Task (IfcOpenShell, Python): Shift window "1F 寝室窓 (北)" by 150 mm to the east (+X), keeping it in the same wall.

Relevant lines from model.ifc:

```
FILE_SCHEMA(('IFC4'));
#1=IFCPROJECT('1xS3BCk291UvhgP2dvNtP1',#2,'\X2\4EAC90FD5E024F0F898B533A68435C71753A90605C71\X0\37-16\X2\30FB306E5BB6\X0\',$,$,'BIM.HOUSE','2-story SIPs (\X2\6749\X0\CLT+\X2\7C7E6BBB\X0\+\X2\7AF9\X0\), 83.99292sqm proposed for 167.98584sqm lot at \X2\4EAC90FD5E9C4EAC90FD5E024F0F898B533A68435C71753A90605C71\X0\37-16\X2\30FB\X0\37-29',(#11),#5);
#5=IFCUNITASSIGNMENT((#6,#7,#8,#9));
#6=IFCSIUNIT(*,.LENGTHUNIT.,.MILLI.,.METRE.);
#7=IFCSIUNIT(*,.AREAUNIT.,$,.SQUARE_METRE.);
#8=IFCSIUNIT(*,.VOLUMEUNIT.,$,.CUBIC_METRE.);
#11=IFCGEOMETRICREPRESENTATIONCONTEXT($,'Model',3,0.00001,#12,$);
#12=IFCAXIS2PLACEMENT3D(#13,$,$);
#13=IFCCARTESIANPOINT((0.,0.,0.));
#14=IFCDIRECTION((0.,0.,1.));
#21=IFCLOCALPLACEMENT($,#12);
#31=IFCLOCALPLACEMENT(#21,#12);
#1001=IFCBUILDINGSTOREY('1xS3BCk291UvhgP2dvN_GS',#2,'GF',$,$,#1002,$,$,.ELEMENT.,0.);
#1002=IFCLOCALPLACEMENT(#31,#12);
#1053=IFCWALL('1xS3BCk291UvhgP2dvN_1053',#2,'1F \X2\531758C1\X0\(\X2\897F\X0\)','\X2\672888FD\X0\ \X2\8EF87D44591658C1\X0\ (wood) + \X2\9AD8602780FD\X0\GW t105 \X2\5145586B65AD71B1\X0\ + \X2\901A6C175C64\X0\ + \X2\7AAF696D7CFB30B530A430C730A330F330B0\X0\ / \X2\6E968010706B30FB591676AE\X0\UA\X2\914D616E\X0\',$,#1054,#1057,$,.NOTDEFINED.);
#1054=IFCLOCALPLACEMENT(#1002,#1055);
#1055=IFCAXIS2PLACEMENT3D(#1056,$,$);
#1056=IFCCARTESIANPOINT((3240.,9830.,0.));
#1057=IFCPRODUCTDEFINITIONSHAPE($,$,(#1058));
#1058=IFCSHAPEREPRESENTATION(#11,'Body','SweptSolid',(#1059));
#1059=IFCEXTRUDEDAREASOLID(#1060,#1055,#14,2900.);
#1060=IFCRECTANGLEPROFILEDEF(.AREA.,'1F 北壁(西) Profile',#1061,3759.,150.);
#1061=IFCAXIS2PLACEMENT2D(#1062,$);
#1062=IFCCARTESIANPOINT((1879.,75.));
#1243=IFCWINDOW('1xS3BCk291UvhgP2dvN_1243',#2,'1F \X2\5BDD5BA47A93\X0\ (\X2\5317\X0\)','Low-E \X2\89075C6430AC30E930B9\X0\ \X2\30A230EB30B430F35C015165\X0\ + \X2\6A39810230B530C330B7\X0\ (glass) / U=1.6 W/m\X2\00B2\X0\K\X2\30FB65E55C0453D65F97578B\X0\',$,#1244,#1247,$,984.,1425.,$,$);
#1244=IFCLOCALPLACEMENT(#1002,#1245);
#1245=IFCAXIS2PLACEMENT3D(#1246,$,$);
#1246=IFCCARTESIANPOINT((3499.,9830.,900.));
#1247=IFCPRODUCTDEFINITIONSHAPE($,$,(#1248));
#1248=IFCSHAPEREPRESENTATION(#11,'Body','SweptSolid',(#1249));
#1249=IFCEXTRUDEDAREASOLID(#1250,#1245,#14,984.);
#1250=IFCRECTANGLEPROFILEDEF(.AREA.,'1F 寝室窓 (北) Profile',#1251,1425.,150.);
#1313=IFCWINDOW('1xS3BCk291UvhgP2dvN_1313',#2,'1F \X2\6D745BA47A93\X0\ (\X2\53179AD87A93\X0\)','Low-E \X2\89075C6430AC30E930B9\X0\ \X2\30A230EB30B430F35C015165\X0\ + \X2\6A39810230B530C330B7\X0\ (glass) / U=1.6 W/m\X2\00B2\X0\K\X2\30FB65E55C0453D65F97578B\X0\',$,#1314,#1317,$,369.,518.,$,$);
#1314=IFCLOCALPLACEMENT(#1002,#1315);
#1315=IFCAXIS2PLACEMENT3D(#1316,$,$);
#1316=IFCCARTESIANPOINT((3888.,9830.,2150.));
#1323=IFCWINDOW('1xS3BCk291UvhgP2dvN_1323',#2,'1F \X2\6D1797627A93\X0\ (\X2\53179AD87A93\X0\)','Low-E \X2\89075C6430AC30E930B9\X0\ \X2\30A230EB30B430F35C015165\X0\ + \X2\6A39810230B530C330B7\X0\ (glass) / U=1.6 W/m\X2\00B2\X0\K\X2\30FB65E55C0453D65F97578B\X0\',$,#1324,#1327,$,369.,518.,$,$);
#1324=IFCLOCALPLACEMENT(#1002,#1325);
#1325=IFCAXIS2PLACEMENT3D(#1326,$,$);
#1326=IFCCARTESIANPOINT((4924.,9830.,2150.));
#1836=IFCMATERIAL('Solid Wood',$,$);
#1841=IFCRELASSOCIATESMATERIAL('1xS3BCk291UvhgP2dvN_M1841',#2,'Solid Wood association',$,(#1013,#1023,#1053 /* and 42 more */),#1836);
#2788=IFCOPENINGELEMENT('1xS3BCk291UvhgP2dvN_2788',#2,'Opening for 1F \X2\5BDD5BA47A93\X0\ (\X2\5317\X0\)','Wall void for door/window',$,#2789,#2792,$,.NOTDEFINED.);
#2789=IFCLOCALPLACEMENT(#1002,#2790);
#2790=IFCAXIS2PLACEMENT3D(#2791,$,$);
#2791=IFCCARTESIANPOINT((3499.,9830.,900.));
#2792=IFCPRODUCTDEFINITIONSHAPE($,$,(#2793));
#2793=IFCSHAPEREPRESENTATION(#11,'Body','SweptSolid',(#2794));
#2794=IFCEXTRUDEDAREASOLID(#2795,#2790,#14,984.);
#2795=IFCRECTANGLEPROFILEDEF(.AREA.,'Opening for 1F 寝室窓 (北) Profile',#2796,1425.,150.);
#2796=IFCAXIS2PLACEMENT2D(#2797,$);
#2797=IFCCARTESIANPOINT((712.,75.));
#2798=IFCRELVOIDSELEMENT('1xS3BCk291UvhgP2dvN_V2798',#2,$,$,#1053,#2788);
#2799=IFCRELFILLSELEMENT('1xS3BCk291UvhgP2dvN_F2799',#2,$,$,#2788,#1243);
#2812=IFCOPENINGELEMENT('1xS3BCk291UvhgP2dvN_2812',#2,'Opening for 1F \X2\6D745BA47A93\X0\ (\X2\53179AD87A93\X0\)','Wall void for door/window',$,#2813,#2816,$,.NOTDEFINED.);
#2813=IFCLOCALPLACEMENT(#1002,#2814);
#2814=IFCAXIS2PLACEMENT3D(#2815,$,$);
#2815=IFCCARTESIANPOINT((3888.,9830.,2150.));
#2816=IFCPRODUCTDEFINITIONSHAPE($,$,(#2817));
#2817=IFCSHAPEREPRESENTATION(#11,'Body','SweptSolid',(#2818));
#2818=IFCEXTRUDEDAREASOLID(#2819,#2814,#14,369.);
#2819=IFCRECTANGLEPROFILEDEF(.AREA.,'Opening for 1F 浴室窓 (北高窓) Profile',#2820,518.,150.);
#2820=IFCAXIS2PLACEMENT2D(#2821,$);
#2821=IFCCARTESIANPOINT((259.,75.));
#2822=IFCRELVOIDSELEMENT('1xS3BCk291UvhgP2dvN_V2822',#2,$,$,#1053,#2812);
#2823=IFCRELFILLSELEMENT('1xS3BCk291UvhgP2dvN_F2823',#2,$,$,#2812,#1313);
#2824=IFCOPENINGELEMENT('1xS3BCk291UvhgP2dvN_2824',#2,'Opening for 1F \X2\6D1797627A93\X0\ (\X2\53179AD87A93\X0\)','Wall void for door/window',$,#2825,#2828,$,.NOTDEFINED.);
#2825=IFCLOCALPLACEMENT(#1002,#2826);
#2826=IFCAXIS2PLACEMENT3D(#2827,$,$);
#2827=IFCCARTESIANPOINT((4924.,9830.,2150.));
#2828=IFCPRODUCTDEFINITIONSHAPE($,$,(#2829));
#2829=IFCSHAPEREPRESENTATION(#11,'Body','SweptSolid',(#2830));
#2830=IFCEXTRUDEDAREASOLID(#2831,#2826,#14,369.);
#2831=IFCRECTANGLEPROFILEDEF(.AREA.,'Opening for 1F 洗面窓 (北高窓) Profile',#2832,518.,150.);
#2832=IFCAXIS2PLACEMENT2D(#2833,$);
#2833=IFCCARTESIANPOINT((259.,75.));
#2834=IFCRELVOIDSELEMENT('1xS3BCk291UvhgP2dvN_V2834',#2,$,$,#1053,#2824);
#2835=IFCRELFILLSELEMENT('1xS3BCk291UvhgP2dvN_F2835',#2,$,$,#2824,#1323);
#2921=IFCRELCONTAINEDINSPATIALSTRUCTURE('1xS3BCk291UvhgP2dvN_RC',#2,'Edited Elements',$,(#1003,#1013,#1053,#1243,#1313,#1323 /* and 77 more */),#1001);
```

```python
import ifcopenshell
import ifcopenshell.api.geometry
import ifcopenshell.util.placement

model = ifcopenshell.open("model.ifc")

window = model.by_guid("1xS3BCk291UvhgP2dvN_1243")
opening = window.FillsVoids[0].RelatingOpeningElement
wall = opening.VoidsElements[0].RelatingBuildingElement

wall_matrix = ifcopenshell.util.placement.get_local_placement(wall.ObjectPlacement)
shift = wall_matrix[:3, 0] * 150.0
before = ifcopenshell.util.placement.get_local_placement(window.ObjectPlacement)[:3, 3].copy()

# The window is not placed relative to its opening, so move both.
for product in (opening, window):
    matrix = ifcopenshell.util.placement.get_local_placement(product.ObjectPlacement)
    matrix[:3, 3] += shift
    ifcopenshell.api.geometry.edit_object_placement(model, product=product, matrix=matrix, is_si=False)

after = ifcopenshell.util.placement.get_local_placement(window.ObjectPlacement)[:3, 3]
print("window moved by", (after - before).round(3) + 0.0)

model.write("model_edited.ifc")
```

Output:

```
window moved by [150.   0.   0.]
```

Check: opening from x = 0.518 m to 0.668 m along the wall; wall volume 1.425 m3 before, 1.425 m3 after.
